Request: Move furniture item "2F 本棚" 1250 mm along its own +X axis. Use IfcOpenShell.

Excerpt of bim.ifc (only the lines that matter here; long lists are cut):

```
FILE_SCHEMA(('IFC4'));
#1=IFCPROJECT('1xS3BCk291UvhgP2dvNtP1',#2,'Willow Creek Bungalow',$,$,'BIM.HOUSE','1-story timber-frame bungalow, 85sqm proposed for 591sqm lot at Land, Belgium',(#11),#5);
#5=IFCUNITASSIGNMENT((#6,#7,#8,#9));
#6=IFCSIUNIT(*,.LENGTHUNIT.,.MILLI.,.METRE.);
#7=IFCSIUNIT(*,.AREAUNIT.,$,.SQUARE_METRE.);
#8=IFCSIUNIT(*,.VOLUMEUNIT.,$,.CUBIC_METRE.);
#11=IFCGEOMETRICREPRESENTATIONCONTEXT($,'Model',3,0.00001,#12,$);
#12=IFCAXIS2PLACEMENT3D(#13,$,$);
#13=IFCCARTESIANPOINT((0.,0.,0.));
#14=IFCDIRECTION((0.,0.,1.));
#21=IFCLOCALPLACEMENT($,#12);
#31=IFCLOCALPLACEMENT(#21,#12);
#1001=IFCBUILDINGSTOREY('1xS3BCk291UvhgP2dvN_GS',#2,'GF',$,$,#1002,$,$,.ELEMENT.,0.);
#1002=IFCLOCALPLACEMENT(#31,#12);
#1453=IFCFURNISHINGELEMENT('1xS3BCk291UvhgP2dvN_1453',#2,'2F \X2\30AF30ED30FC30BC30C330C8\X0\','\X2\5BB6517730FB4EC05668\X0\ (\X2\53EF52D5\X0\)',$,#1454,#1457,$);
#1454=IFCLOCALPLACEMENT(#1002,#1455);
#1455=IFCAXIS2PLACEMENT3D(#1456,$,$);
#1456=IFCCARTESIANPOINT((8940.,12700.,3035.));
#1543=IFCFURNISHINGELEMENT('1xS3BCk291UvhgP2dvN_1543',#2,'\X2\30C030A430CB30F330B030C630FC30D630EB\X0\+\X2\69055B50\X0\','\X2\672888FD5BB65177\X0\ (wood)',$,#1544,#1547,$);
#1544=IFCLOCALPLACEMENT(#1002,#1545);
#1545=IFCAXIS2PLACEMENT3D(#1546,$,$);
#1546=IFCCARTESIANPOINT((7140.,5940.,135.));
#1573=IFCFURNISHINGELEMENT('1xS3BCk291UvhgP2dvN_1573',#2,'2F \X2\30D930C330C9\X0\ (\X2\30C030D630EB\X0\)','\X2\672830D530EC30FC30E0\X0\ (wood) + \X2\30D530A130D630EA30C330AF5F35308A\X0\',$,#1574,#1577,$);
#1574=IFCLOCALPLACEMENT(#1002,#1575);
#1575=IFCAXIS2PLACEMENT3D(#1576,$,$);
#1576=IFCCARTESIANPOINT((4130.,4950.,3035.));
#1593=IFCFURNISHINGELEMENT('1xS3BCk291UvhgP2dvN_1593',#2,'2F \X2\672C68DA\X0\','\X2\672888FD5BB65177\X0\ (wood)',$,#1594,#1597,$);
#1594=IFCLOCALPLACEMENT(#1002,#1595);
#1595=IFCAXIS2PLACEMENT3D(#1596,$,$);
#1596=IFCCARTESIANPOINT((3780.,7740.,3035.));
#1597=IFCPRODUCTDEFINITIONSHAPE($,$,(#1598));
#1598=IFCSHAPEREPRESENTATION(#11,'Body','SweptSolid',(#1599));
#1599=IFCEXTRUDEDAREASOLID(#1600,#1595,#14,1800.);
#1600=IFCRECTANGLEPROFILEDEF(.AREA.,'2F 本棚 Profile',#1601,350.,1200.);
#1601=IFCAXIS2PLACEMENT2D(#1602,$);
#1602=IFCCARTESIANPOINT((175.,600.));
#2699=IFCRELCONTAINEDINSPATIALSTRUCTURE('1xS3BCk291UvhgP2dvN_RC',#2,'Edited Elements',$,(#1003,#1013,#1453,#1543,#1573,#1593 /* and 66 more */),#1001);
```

```python
import ifcopenshell
import ifcopenshell.api.geometry
import ifcopenshell.util.placement
import ifcopenshell.util.unit

model = ifcopenshell.open("bim.ifc")
unit_scale = ifcopenshell.util.unit.calculate_unit_scale(model)

item = model.by_id(1593)
matrix = ifcopenshell.util.placement.get_local_placement(item.ObjectPlacement)
matrix[:3, 3] += matrix[:3, 0] * 1.25 / unit_scale
ifcopenshell.api.geometry.edit_object_placement(model, product=item, matrix=matrix, is_si=False)

print(ifcopenshell.util.placement.get_local_placement(item.ObjectPlacement).round(3) + 0.0)

model.write("bim-out.ifc")
```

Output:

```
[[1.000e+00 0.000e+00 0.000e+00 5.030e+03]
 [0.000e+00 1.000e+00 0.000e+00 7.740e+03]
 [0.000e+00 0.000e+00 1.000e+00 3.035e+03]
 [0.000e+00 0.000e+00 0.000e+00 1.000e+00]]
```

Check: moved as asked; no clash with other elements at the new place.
